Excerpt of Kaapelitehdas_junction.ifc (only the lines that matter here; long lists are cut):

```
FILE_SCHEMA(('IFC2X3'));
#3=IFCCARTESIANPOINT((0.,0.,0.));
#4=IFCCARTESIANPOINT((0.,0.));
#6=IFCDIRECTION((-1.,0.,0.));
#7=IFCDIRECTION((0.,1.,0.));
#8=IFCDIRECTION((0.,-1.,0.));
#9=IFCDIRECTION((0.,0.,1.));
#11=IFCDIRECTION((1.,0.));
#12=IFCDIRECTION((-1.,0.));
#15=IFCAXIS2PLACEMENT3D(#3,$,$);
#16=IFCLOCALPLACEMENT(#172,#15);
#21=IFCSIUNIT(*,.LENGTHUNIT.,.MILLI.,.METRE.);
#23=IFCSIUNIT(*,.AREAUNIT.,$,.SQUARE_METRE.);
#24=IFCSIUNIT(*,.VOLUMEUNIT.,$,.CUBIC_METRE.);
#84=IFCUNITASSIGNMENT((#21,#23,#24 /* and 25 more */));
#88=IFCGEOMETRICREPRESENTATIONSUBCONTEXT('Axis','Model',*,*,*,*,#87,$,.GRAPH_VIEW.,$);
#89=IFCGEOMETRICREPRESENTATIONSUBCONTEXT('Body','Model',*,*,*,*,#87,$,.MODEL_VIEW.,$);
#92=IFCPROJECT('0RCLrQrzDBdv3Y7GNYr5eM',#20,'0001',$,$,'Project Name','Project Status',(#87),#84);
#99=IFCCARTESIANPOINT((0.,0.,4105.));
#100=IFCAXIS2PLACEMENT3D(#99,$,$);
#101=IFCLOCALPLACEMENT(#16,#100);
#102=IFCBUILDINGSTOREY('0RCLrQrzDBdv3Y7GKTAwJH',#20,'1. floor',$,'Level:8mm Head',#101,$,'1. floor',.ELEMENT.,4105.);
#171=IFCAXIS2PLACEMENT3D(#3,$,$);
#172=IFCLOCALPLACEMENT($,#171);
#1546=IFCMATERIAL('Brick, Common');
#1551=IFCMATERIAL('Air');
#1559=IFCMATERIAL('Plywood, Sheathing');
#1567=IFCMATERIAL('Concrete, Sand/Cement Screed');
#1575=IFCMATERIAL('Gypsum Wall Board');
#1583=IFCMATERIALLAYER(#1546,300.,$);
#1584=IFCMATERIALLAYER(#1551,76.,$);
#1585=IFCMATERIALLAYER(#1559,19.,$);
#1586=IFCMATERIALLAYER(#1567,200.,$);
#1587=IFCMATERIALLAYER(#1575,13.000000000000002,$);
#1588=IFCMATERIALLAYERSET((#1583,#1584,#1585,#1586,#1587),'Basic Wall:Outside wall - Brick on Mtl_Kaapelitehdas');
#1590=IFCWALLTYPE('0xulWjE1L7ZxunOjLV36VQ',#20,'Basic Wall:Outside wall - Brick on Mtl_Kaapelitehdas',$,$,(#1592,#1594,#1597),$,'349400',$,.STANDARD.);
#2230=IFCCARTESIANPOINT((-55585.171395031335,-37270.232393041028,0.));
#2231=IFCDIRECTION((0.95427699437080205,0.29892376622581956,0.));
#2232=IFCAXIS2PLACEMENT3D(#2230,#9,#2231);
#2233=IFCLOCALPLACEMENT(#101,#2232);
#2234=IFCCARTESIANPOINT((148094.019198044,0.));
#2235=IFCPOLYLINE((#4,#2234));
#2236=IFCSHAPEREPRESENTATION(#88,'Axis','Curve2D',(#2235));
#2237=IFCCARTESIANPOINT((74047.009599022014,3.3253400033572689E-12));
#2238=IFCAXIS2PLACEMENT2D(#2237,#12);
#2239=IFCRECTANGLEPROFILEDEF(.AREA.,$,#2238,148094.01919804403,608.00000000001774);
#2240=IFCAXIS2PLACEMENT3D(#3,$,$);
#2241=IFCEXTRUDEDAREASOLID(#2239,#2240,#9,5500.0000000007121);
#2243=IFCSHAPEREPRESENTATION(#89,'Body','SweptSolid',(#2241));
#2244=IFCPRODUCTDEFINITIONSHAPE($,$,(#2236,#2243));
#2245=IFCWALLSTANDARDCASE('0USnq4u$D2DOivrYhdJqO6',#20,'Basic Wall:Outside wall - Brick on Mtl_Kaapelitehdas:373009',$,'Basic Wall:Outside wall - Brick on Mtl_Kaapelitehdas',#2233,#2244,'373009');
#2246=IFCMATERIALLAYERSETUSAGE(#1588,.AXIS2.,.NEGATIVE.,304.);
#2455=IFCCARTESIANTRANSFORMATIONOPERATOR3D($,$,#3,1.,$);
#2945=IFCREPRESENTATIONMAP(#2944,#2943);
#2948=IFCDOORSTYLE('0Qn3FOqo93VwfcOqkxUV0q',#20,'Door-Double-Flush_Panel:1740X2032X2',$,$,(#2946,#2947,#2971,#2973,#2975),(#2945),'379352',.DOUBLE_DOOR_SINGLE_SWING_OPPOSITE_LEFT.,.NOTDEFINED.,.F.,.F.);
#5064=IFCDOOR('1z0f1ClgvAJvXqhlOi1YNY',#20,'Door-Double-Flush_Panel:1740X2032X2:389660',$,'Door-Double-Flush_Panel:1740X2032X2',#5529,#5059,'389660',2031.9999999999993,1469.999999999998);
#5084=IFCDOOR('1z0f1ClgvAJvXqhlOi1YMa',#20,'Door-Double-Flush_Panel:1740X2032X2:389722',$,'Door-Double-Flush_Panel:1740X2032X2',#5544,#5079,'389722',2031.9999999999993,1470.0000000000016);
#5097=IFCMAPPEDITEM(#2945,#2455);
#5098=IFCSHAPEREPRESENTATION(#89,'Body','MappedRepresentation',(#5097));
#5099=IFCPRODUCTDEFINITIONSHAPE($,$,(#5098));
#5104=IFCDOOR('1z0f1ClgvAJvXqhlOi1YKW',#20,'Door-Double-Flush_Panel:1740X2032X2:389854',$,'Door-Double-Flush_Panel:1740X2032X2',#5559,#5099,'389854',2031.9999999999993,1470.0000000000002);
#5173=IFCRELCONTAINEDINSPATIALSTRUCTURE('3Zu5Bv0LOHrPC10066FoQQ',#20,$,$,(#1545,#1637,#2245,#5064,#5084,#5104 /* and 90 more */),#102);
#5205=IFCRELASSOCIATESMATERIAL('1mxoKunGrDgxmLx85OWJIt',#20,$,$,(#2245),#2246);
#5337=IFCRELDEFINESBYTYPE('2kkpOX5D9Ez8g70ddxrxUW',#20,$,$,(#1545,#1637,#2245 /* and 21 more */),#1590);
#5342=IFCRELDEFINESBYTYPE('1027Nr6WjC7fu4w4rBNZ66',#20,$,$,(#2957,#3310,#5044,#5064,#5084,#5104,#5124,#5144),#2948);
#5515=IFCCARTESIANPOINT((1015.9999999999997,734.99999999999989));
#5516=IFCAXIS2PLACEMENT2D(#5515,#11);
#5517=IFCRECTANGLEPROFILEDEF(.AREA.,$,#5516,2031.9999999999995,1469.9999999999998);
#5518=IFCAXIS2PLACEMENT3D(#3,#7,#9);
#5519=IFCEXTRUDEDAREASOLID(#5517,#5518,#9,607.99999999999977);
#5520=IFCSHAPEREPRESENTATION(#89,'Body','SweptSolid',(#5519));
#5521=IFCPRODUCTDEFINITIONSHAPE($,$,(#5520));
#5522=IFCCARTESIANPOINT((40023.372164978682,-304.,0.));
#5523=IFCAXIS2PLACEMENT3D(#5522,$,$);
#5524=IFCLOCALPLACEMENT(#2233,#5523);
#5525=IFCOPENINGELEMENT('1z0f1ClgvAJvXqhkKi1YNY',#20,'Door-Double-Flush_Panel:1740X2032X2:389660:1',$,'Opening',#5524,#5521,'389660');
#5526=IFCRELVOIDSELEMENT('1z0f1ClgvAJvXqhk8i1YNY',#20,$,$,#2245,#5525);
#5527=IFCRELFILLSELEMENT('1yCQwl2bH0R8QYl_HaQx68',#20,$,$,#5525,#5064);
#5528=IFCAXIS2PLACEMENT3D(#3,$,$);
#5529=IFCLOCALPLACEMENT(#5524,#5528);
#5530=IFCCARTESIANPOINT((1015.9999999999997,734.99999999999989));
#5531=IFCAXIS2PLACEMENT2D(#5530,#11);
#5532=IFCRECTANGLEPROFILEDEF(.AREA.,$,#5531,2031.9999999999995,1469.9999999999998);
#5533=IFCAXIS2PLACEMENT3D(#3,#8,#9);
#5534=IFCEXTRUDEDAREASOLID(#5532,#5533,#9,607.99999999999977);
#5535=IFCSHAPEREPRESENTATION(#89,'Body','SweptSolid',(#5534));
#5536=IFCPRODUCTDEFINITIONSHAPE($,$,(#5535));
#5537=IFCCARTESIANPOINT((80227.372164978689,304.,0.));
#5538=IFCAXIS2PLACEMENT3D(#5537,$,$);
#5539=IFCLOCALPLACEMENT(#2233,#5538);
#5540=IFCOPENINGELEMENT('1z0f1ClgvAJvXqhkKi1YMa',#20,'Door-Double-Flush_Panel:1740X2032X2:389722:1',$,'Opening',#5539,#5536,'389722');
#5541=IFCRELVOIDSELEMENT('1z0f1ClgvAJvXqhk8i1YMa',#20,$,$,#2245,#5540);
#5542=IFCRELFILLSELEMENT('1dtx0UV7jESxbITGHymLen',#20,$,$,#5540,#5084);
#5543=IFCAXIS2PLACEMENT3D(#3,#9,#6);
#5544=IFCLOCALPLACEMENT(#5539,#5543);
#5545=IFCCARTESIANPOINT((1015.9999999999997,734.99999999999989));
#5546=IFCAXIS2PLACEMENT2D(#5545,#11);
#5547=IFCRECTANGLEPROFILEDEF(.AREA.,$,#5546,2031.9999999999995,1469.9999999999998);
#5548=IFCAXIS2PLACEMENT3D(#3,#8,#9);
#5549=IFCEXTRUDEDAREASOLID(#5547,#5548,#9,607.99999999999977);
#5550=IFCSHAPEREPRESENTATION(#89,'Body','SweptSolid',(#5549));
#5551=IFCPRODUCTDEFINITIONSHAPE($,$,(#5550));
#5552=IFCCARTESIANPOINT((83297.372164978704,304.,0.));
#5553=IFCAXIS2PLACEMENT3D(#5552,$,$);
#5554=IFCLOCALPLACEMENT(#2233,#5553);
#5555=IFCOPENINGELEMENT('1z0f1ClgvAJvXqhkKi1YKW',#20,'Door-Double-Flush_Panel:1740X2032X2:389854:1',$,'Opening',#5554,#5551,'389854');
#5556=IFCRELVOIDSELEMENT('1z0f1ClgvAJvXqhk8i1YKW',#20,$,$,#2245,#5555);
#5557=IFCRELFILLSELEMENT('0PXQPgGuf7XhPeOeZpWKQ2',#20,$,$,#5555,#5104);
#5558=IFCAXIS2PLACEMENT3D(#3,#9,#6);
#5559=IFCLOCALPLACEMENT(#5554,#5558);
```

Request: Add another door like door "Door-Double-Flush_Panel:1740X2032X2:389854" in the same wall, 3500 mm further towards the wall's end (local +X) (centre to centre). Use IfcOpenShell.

```python
import ifcopenshell
import ifcopenshell.api.feature
import ifcopenshell.api.geometry
import ifcopenshell.api.root
import ifcopenshell.geom
import ifcopenshell.util.element
import ifcopenshell.util.placement
import ifcopenshell.util.shape

model = ifcopenshell.open("Kaapelitehdas_junction.ifc")
settings = ifcopenshell.geom.settings()


def volume(element):
    """Net volume in cubic metres, openings subtracted."""
    shape = ifcopenshell.geom.create_shape(settings, element)
    return ifcopenshell.util.shape.get_volume(shape.geometry)


def reuse_history(source, copy):
    """copy_class also copies each property set's owner history, people and application; keep the originals."""
    for rel in copy.IsDefinedBy:
        if rel.is_a("IfcRelDefinesByProperties") and (history := rel.RelatingPropertyDefinition.OwnerHistory):
            rel.RelatingPropertyDefinition.OwnerHistory = source.OwnerHistory
            ifcopenshell.util.element.remove_deep2(model, history)


door = model.by_guid("1z0f1ClgvAJvXqhlOi1YKW")
opening = door.FillsVoids[0].RelatingOpeningElement
wall = opening.VoidsElements[0].RelatingBuildingElement
before = volume(wall)
shift = ifcopenshell.util.placement.get_local_placement(wall.ObjectPlacement)[:3, 0] * 3500.0

# copy_class copies the void relationship, type, container and properties, but no geometry.
new_opening = ifcopenshell.api.root.copy_class(model, product=opening)
new_opening.Representation = ifcopenshell.util.element.copy_deep(
    model, opening.Representation, exclude=["IfcGeometricRepresentationContext", "IfcRepresentationMap"]
)
new_opening.Name = "Door-Double-Flush_Panel:1740X2032X2"
new_opening.Tag = None
new_door = ifcopenshell.api.root.copy_class(model, product=door)
new_door.Representation = ifcopenshell.util.element.copy_deep(
    model, door.Representation, exclude=["IfcGeometricRepresentationContext", "IfcRepresentationMap"]
)
new_door.Name = "Door-Double-Flush_Panel:1740X2032X2"
new_door.Tag = None
reuse_history(door, new_door)
fills = ifcopenshell.api.feature.add_filling(model, opening=new_opening, element=new_door)
fills.OwnerHistory = new_door.OwnerHistory  # required in IFC2X3

for old, new in ((opening, new_opening), (door, new_door)):
    matrix = ifcopenshell.util.placement.get_local_placement(old.ObjectPlacement)
    matrix[:3, 3] += shift
    ifcopenshell.api.geometry.edit_object_placement(model, product=new, matrix=matrix, is_si=False)

after = volume(wall)

print(f"wall volume {before:.3f} -> {after:.3f} m3")

model.write("Kaapelitehdas_junction_edited.ifc")
```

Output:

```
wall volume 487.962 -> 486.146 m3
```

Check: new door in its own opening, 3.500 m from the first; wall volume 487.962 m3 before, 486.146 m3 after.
